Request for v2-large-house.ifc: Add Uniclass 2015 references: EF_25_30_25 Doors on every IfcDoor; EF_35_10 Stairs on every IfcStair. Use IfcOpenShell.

First a look at what the model holds.

```python
import ifcopenshell

model = ifcopenshell.open("v2-large-house.ifc")
print(model.schema)
print("classifications:", [c.Name for c in model.by_type("IfcClassification")])
for ifc_class in ("IfcDoor", "IfcRoof", "IfcStair", "IfcWall", "IfcWindow"):
    print(ifc_class, len(model.by_type(ifc_class)))
```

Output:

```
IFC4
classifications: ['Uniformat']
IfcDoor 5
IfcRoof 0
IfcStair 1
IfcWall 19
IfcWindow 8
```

```python
import ifcopenshell
import ifcopenshell.api.classification

model = ifcopenshell.open("v2-large-house.ifc")

system = ifcopenshell.api.classification.add_classification(model, classification="Uniclass 2015")

codes = {
    "IfcDoor": ("EF_25_30_25", "Doors"),
    "IfcStair": ("EF_35_10", "Stairs"),
}
for ifc_class, (code, name) in codes.items():
    products = model.by_type(ifc_class)
    ifcopenshell.api.classification.add_reference(
        model, products=products, classification=system, identification=code, name=name
    )
    print(code, len(products))

model.write("v2-large-house_updated.ifc")
```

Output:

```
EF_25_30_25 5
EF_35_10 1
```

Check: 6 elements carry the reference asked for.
